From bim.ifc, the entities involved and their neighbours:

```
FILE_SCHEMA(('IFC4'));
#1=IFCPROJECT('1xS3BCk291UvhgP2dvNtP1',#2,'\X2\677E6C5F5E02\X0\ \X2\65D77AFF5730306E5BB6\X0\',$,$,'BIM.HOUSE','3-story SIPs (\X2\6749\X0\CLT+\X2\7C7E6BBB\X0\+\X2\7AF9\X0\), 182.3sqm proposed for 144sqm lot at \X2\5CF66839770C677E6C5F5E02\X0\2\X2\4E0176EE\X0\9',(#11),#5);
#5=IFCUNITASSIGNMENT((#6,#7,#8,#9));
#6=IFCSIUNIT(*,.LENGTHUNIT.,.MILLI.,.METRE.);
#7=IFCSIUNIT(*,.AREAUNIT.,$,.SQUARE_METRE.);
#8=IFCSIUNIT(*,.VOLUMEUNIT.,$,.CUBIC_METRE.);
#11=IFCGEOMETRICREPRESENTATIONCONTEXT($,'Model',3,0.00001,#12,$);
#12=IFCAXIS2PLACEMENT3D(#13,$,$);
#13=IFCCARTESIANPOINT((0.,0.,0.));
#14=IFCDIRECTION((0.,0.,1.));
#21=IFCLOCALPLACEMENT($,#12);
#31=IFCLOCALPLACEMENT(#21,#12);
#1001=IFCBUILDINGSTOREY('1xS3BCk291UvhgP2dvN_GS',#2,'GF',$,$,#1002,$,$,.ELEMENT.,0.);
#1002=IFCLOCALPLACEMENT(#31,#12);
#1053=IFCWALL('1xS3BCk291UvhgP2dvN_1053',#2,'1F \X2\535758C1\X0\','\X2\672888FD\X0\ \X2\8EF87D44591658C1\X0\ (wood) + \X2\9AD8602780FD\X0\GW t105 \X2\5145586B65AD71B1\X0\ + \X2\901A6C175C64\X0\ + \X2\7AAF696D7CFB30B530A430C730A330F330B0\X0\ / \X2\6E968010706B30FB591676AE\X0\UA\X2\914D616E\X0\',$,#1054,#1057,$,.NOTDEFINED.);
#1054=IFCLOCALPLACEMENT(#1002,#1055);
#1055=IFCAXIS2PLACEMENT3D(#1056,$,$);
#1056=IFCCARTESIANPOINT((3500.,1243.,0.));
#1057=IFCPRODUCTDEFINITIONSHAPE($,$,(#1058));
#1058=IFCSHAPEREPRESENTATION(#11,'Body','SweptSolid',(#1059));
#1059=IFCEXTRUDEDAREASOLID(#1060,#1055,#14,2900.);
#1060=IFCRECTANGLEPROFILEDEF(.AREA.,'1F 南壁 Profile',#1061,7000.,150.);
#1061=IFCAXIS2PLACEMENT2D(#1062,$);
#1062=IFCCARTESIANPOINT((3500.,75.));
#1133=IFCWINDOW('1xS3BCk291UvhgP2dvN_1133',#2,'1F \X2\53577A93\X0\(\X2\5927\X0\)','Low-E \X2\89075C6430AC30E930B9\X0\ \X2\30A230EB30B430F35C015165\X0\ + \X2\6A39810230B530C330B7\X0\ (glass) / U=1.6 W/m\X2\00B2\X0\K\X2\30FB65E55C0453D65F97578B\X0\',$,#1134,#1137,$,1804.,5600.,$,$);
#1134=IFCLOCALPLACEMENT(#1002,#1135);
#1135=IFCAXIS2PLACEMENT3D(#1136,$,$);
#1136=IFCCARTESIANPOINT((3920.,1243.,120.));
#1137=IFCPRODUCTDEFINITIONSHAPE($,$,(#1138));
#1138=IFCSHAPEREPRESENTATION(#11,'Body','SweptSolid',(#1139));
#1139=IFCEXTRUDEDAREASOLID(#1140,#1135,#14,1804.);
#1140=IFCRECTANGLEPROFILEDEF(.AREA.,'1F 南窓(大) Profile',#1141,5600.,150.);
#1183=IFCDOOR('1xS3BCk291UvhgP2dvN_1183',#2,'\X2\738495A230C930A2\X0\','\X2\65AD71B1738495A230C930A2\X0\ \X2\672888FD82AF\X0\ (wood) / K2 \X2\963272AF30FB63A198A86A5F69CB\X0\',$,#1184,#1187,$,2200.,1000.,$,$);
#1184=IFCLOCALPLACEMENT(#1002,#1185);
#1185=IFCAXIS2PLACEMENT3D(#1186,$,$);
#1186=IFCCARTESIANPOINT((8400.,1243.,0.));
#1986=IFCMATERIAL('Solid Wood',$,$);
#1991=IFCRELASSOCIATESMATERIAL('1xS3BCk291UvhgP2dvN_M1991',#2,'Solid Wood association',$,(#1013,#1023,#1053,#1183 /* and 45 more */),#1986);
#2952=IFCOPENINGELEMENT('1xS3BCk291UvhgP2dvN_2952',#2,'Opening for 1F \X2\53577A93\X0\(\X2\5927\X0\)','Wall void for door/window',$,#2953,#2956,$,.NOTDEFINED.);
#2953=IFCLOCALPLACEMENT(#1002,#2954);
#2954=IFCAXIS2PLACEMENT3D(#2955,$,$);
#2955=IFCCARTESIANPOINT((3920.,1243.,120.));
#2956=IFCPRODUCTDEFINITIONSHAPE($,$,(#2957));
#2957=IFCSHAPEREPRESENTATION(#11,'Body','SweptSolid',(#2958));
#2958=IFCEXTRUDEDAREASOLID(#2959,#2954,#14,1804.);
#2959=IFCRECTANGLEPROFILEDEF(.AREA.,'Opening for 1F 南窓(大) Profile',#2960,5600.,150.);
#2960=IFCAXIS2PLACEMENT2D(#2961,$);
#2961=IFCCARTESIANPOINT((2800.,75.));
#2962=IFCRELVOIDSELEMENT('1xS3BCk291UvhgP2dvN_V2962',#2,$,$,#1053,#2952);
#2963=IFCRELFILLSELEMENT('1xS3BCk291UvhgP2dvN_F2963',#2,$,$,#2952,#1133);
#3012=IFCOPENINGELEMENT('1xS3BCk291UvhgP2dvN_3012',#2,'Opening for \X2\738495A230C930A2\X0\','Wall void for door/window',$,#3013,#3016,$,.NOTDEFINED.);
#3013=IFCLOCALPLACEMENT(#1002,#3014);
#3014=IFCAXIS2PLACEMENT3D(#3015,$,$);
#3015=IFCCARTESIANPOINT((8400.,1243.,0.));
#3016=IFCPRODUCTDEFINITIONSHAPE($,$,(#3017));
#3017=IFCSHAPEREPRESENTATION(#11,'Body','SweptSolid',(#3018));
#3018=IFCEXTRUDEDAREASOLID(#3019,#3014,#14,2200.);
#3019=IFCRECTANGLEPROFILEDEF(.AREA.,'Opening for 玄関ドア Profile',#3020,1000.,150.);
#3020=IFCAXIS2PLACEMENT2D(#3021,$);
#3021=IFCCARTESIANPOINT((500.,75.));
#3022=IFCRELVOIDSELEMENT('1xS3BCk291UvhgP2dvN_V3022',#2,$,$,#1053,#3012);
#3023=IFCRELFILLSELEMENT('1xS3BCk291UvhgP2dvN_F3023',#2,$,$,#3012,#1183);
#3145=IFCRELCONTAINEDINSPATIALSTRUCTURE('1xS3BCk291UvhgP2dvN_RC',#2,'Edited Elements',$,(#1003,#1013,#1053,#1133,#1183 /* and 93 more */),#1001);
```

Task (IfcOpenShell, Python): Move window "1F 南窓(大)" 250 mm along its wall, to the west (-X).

```python
import ifcopenshell
import ifcopenshell.api.geometry
import ifcopenshell.util.placement

model = ifcopenshell.open("bim.ifc")

window = model.by_guid("1xS3BCk291UvhgP2dvN_1133")
opening = window.FillsVoids[0].RelatingOpeningElement
wall = opening.VoidsElements[0].RelatingBuildingElement

wall_matrix = ifcopenshell.util.placement.get_local_placement(wall.ObjectPlacement)
shift = wall_matrix[:3, 0] * -250.0
before = ifcopenshell.util.placement.get_local_placement(window.ObjectPlacement)[:3, 3].copy()

# The window is not placed relative to its opening, so move both.
for product in (opening, window):
    matrix = ifcopenshell.util.placement.get_local_placement(product.ObjectPlacement)
    matrix[:3, 3] += shift
    ifcopenshell.api.geometry.edit_object_placement(model, product=product, matrix=matrix, is_si=False)

after = ifcopenshell.util.placement.get_local_placement(window.ObjectPlacement)[:3, 3]
print("window moved by", (after - before).round(3) + 0.0)

model.write("bim_rev.ifc")
```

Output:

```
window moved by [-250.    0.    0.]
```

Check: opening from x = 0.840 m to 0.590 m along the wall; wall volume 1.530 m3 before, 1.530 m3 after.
